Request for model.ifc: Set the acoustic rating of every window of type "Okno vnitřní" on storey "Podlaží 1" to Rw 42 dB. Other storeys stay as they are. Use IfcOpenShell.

First a look at what the model holds.

```python
import ifcopenshell
import ifcopenshell.util.element

model = ifcopenshell.open("model.ifc")
print(model.schema)
storey = next(s for s in model.by_type("IfcBuildingStorey") if s.Name == "Podlaží 1")
windows = [e for e in ifcopenshell.util.element.get_decomposition(storey) if e.is_a("IfcWindow")]
seen = {}
for e in windows:
    element_type = ifcopenshell.util.element.get_type(e)
    key = (element_type.Name if element_type != e and element_type else None, ifcopenshell.util.element.get_pset(e, "Pset_WindowCommon", "AcousticRating"))
    seen[key] = seen.get(key, 0) + 1
for (name, value), count in sorted(seen.items(), key=str):
    print(count, "x", name, "|", value)
```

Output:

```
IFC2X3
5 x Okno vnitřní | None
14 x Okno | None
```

```python
import ifcopenshell
import ifcopenshell.api.pset
import ifcopenshell.util.element

model = ifcopenshell.open("model.ifc")

storey = next(s for s in model.by_type("IfcBuildingStorey") if s.Name == "Podlaží 1")
windows = [e for e in ifcopenshell.util.element.get_decomposition(storey) if e.is_a("IfcWindow")]

count = 0
for e in windows:
    element_type = ifcopenshell.util.element.get_type(e)
    if element_type in (None, e) or element_type.Name != "Okno vnitřní":
        continue
    # add_pset returns the element's existing set when there is one.
    pset = ifcopenshell.api.pset.add_pset(model, product=e, name="Pset_WindowCommon")
    ifcopenshell.api.pset.edit_pset(model, pset=pset, properties={"AcousticRating": "Rw 42 dB"})
    count += 1

print(count, "windows updated")

model.write("model-out.ifc")
```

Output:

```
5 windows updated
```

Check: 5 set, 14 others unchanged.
